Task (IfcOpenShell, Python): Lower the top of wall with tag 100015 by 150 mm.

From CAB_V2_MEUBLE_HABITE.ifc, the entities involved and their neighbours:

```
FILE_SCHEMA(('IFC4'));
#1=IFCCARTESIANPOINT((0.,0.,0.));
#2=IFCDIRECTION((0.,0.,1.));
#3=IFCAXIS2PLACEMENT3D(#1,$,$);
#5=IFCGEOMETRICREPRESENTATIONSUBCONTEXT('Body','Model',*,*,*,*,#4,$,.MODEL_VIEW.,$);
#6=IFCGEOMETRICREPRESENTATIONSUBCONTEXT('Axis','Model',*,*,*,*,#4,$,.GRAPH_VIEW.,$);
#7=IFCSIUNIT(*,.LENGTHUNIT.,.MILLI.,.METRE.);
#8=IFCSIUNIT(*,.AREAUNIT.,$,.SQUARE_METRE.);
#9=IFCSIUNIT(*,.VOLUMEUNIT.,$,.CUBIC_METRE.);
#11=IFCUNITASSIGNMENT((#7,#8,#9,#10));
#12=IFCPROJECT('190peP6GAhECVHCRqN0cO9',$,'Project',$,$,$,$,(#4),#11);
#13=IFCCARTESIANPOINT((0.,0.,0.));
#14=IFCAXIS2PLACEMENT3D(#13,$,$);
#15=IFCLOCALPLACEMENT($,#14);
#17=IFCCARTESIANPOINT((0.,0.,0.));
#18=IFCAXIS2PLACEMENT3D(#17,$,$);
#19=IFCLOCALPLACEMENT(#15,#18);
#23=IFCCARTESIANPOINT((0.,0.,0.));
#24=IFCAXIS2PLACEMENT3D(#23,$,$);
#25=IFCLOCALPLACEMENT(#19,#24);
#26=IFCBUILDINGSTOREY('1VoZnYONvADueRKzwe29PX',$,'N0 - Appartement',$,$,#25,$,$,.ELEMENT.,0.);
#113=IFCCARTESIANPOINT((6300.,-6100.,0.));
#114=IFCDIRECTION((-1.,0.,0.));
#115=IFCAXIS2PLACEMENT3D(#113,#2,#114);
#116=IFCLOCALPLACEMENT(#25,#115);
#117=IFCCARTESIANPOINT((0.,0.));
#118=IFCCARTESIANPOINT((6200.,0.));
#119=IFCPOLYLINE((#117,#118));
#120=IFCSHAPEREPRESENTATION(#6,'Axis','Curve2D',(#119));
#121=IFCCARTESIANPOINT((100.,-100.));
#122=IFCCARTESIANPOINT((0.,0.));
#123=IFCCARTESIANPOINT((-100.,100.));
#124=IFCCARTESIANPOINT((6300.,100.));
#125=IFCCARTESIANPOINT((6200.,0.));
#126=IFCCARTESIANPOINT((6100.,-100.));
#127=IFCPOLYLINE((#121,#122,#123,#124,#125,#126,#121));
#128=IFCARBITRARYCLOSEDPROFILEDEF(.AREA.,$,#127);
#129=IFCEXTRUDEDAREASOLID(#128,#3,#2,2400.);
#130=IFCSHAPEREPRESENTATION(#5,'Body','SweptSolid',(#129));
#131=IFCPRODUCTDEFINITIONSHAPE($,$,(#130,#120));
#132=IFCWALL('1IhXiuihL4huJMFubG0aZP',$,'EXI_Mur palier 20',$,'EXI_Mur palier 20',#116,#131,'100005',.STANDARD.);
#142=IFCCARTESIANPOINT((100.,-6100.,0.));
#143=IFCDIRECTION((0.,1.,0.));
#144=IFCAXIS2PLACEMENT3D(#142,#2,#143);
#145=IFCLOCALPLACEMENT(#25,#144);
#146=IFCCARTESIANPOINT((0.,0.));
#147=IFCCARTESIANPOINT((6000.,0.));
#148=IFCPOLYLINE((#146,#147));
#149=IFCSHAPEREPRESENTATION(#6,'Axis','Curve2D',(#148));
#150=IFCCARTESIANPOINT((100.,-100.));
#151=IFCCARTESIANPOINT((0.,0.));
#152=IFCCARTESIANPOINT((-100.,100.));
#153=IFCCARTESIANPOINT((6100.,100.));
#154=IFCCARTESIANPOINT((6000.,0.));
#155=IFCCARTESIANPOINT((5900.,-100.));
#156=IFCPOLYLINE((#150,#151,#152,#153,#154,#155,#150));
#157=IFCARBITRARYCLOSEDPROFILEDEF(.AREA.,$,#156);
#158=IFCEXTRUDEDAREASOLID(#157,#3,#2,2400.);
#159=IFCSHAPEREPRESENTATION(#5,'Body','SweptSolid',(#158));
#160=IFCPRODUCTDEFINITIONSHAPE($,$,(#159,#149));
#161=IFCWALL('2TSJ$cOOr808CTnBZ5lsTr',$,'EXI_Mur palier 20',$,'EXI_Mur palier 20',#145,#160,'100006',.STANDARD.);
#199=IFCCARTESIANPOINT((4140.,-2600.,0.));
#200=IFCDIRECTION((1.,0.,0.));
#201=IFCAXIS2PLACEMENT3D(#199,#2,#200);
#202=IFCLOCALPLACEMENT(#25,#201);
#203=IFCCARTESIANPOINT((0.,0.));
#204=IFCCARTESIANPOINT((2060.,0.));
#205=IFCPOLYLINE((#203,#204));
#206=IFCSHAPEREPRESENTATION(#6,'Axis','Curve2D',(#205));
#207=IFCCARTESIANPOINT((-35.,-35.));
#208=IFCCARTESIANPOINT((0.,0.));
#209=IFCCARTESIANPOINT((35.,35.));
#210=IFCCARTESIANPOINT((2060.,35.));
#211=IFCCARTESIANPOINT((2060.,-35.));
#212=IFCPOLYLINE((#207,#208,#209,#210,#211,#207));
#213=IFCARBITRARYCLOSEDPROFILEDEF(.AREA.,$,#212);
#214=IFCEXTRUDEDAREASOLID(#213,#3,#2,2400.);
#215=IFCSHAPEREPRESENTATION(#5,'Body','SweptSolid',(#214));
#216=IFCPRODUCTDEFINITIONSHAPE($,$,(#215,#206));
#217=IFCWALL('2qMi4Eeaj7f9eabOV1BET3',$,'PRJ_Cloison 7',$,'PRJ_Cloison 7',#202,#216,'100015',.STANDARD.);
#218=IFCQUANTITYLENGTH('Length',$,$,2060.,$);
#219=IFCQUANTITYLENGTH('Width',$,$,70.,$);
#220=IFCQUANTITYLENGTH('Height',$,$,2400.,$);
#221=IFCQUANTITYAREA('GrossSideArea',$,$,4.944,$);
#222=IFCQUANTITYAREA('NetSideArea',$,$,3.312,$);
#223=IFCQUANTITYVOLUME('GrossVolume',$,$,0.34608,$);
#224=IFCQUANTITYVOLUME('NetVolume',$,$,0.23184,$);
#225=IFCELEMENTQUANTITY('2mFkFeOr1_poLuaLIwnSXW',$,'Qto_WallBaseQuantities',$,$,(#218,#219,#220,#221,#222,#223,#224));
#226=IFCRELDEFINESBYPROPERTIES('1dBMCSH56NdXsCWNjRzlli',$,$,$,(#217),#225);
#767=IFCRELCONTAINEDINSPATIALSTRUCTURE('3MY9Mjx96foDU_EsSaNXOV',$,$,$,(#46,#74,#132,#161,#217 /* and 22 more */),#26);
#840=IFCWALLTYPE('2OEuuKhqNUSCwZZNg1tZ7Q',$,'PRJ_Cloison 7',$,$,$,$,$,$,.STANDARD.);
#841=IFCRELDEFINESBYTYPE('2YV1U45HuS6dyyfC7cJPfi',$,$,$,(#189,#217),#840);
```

```python
import ifcopenshell
import ifcopenshell.api.pset
import ifcopenshell.geom
import ifcopenshell.util.element
import ifcopenshell.util.representation
import ifcopenshell.util.shape
import ifcopenshell.util.unit

model = ifcopenshell.open("CAB_V2_MEUBLE_HABITE.ifc")
unit_scale = ifcopenshell.util.unit.calculate_unit_scale(model)
area_scale = ifcopenshell.util.unit.calculate_unit_scale(model, "AREAUNIT")
volume_scale = ifcopenshell.util.unit.calculate_unit_scale(model, "VOLUMEUNIT")
settings = ifcopenshell.geom.settings()


def volume(element):
    """Net volume in cubic metres, openings subtracted."""
    shape = ifcopenshell.geom.create_shape(settings, element)
    return ifcopenshell.util.shape.get_volume(shape.geometry)


wall = model.by_guid("2qMi4Eeaj7f9eabOV1BET3")
before = volume(wall)

body = ifcopenshell.util.representation.get_representation(wall, "Model", "Body")
solid = body.Items[0]
old_height = solid.Depth
solid.Depth -= 150.0
after = volume(wall)
thickness = 0.07  # wall thickness in metres

# Update the stored height, areas and volumes.
qto = model.by_id(ifcopenshell.util.element.get_pset(wall, "Qto_WallBaseQuantities", should_inherit=False)["id"])
ifcopenshell.api.pset.edit_qto(model, qto=qto, properties={
    "Height": solid.Depth,
    "GrossSideArea": ifcopenshell.util.element.get_pset(wall, "Qto_WallBaseQuantities", "GrossSideArea") * solid.Depth / old_height,
    "NetSideArea": after / thickness / area_scale,
    "GrossVolume": ifcopenshell.util.element.get_pset(wall, "Qto_WallBaseQuantities", "GrossVolume") * solid.Depth / old_height,
    "NetVolume": after / volume_scale,
})

print(f"height {old_height:g} -> {solid.Depth:g}, volume {before:.3f} -> {after:.3f} m3")

model.write("CAB_V2_MEUBLE_HABITE_updated.ifc")
```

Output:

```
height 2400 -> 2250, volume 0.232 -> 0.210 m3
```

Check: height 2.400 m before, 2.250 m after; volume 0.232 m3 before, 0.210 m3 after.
